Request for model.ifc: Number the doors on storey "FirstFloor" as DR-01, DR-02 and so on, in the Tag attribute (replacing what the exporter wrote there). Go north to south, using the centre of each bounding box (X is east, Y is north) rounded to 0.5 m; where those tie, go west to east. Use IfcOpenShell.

First a look at what the model holds.

```python
import ifcopenshell
import ifcopenshell.util.element
import ifcopenshell.util.placement

model = ifcopenshell.open("model.ifc")
print(model.schema)
storey = next(s for s in model.by_type("IfcBuildingStorey") if s.Name == "FirstFloor")
doors = [e for e in ifcopenshell.util.element.get_decomposition(storey) if e.is_a("IfcDoor")]
for e in sorted(doors, key=lambda e: e.id()):
    origin = ifcopenshell.util.placement.get_local_placement(e.ObjectPlacement)[:3, 3]
    print(e.id(), e.Tag, e.Name, origin.round(2) + 0.0, sep=" | ")
```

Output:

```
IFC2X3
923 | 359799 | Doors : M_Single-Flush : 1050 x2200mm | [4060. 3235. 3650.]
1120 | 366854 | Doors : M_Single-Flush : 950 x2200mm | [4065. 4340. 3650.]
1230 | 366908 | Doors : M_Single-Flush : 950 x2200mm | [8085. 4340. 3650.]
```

```python
import ifcopenshell
import ifcopenshell.geom
import ifcopenshell.util.element
import ifcopenshell.util.shape

model = ifcopenshell.open("model.ifc")
settings = ifcopenshell.geom.settings()
settings.set("use-world-coords", True)


def centre(element):
    shape = ifcopenshell.geom.create_shape(settings, element)
    return ifcopenshell.util.shape.get_bbox_centroid(shape.geometry)


storey = next(s for s in model.by_type("IfcBuildingStorey") if s.Name == "FirstFloor")
doors = [e for e in ifcopenshell.util.element.get_decomposition(storey) if e.is_a("IfcDoor")]

# Insertion points can sit at a corner or the storey origin, so sort by the geometry (in metres).
centres = {e: centre(e) for e in doors}
doors.sort(key=lambda e: (-round(centres[e][1] / 0.5), centres[e][0]))

for i, e in enumerate(doors, start=1):
    number = f"DR-{i:02d}"
    e.Tag = number
    print(e.id(), number)

model.write("model-out.ifc")
```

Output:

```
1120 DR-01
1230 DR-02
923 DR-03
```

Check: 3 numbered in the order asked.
